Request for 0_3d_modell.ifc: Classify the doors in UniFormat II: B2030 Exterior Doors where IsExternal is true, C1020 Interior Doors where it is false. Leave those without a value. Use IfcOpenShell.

First a look at what the model holds.

```python
import ifcopenshell
import ifcopenshell.util.element

model = ifcopenshell.open("0_3d_modell.ifc")
print(model.schema)
print("classifications:", [c.Name for c in model.by_type("IfcClassification")])
values = [ifcopenshell.util.element.get_pset(e, "Pset_DoorCommon", "IsExternal") for e in model.by_type("IfcDoor")]
for value in (True, False, None):
    print("IsExternal", value, values.count(value))
```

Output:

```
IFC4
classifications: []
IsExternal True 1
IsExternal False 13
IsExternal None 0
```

```python
import ifcopenshell
import ifcopenshell.api.classification
import ifcopenshell.util.element

model = ifcopenshell.open("0_3d_modell.ifc")

system = ifcopenshell.api.classification.add_classification(model, classification="UniFormat II")

doors = model.by_type("IfcDoor")
external = {e: ifcopenshell.util.element.get_pset(e, "Pset_DoorCommon", "IsExternal") for e in doors}
for flag, code, name in ((True, "B2030", "Exterior Doors"), (False, "C1020", "Interior Doors")):
    products = [e for e in doors if external[e] is flag]
    ifcopenshell.api.classification.add_reference(
        model, products=products, classification=system, identification=code, name=name
    )
    print(code, len(products))

model.write("0_3d_modell-out.ifc")
```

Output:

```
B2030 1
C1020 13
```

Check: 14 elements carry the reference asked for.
